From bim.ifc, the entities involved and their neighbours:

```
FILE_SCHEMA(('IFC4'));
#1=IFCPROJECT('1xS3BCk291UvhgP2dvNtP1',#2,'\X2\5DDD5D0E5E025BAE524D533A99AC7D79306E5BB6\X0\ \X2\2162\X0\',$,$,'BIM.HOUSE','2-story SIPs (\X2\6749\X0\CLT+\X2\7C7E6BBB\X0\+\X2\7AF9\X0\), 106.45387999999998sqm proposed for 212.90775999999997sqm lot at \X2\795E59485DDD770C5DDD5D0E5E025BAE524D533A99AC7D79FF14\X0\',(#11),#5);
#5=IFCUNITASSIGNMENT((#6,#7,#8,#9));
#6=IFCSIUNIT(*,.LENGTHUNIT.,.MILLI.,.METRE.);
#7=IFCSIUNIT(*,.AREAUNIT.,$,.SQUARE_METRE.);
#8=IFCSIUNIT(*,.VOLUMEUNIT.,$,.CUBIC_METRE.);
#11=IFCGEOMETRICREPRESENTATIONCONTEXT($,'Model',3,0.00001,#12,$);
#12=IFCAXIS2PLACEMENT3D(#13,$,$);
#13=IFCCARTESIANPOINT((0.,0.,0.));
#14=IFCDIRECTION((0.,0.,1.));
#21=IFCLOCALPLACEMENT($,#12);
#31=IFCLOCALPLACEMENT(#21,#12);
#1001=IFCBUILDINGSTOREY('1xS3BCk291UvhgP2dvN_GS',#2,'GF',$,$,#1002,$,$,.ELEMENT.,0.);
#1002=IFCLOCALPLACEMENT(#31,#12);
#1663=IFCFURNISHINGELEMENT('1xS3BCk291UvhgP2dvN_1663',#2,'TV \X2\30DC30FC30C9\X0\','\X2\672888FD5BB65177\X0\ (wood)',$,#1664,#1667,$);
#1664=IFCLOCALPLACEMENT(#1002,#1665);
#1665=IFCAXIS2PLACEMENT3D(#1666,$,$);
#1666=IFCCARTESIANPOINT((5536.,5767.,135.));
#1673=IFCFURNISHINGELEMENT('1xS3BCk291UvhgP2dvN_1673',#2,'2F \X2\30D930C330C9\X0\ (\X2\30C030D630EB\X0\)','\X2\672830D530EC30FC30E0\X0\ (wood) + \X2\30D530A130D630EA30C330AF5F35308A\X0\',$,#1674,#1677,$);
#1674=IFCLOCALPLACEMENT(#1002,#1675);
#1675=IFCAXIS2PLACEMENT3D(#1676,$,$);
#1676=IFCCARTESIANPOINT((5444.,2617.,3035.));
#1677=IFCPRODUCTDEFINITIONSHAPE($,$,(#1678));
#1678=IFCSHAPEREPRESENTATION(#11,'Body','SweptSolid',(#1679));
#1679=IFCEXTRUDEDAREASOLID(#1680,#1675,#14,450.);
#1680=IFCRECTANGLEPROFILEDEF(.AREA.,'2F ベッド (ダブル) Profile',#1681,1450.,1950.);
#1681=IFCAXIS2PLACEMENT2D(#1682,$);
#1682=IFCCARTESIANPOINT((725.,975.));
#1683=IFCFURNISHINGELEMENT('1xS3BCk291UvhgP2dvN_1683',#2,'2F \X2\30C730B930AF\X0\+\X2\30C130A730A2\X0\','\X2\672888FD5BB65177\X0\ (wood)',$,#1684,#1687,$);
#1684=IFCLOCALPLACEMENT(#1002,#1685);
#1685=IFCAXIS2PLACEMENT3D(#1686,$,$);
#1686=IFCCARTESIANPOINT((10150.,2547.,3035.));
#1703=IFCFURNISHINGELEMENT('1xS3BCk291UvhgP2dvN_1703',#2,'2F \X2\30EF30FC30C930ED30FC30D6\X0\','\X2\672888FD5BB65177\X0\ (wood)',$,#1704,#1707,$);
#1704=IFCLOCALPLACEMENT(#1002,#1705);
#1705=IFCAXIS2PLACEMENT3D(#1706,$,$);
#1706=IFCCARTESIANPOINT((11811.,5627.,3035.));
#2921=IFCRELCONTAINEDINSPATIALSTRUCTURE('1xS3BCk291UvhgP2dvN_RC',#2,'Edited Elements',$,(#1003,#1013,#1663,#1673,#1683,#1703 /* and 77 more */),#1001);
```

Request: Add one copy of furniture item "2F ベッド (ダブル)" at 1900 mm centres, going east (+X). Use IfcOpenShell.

```python
import numpy as np
import ifcopenshell
import ifcopenshell.api.geometry
import ifcopenshell.api.root
import ifcopenshell.util.element
import ifcopenshell.util.placement
import ifcopenshell.util.unit

model = ifcopenshell.open("bim.ifc")
unit_scale = ifcopenshell.util.unit.calculate_unit_scale(model)


def reuse_history(source, copy):
    """copy_class also copies each property set's owner history, people and application; keep the originals."""
    for rel in copy.IsDefinedBy:
        if rel.is_a("IfcRelDefinesByProperties") and (history := rel.RelatingPropertyDefinition.OwnerHistory):
            rel.RelatingPropertyDefinition.OwnerHistory = source.OwnerHistory
            ifcopenshell.util.element.remove_deep2(model, history)


source = model.by_guid("1xS3BCk291UvhgP2dvN_1673")
base = ifcopenshell.util.placement.get_local_placement(source.ObjectPlacement)
step = np.array([1.0, 0.0, 0.0]) * 1.9 / unit_scale

for i in range(1, 2):
    copy = ifcopenshell.api.root.copy_class(model, product=source)
    copy.Representation = ifcopenshell.util.element.copy_deep(
        model, source.Representation, exclude=["IfcGeometricRepresentationContext", "IfcRepresentationMap"]
    )
    reuse_history(source, copy)
    matrix = base.copy()
    matrix[:3, 3] += i * step
    print("added at", matrix[:3, 3].round(3) + 0.0)
    ifcopenshell.api.geometry.edit_object_placement(model, product=copy, matrix=matrix, is_si=False)

model.write("bim-out.ifc")
```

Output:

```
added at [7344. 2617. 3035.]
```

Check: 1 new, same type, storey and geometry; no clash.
